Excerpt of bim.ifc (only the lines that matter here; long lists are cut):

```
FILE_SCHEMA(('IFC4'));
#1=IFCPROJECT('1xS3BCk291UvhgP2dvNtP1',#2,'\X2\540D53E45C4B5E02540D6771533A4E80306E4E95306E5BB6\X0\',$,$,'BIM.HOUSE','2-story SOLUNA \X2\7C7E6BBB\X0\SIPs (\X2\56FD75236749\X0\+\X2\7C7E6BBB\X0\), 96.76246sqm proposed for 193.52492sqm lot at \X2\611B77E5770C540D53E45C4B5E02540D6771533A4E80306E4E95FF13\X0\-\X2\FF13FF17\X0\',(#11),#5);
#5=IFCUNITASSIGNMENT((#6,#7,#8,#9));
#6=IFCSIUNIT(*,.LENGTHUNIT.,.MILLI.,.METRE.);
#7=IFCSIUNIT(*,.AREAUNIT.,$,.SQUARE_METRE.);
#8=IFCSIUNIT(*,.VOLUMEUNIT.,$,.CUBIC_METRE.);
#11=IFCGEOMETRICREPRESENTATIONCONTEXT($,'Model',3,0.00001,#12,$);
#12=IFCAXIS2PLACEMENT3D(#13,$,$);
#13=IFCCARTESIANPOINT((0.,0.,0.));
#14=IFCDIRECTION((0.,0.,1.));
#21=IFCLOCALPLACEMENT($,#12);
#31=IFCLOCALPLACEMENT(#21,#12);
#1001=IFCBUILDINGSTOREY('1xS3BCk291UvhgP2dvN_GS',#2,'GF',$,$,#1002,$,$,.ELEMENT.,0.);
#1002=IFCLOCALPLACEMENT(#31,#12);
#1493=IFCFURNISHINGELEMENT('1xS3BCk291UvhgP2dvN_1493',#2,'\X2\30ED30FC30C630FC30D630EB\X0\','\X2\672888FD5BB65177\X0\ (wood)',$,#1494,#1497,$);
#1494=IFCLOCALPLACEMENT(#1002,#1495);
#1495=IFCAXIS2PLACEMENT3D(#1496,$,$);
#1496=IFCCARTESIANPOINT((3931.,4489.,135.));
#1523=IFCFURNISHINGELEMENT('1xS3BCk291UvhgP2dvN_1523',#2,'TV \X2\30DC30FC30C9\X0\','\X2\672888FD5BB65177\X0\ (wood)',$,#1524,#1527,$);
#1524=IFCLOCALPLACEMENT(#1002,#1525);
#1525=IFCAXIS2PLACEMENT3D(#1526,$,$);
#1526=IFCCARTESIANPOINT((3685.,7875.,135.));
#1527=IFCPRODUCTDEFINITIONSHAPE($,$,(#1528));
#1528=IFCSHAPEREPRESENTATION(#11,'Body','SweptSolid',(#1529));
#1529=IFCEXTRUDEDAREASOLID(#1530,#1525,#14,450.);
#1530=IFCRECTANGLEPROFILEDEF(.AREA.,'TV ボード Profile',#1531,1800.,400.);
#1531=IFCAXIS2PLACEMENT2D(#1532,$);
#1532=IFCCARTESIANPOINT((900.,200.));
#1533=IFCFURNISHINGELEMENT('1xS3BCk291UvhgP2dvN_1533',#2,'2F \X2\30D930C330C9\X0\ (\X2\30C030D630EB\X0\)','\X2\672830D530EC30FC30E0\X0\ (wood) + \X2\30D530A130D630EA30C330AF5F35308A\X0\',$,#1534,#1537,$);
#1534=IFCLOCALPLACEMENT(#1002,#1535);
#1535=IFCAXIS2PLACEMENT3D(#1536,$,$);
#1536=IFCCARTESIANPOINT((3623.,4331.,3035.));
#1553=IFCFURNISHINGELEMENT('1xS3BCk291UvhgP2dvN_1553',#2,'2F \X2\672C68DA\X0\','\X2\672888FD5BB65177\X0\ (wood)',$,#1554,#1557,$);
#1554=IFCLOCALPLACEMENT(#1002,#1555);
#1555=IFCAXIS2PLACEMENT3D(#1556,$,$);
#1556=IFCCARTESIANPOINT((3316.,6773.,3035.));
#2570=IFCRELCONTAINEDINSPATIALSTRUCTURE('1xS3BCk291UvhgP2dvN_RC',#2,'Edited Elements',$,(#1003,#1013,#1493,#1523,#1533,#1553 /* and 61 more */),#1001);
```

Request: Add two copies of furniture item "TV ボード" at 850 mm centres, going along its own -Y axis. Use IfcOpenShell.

```python
import ifcopenshell
import ifcopenshell.api.geometry
import ifcopenshell.api.root
import ifcopenshell.util.element
import ifcopenshell.util.placement
import ifcopenshell.util.unit

model = ifcopenshell.open("bim.ifc")
unit_scale = ifcopenshell.util.unit.calculate_unit_scale(model)


def reuse_history(source, copy):
    """copy_class also copies each property set's owner history, people and application; keep the originals."""
    for rel in copy.IsDefinedBy:
        if rel.is_a("IfcRelDefinesByProperties") and (history := rel.RelatingPropertyDefinition.OwnerHistory):
            rel.RelatingPropertyDefinition.OwnerHistory = source.OwnerHistory
            ifcopenshell.util.element.remove_deep2(model, history)


source = model.by_guid("1xS3BCk291UvhgP2dvN_1523")
base = ifcopenshell.util.placement.get_local_placement(source.ObjectPlacement)
step = -base[:3, 1] * 0.85 / unit_scale

for i in range(1, 3):
    copy = ifcopenshell.api.root.copy_class(model, product=source)
    copy.Representation = ifcopenshell.util.element.copy_deep(
        model, source.Representation, exclude=["IfcGeometricRepresentationContext", "IfcRepresentationMap"]
    )
    reuse_history(source, copy)
    matrix = base.copy()
    matrix[:3, 3] += i * step
    print("added at", matrix[:3, 3].round(3) + 0.0)
    ifcopenshell.api.geometry.edit_object_placement(model, product=copy, matrix=matrix, is_si=False)

model.write("bim_updated.ifc")
```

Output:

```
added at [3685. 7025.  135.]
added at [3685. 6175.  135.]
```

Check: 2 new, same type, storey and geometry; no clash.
